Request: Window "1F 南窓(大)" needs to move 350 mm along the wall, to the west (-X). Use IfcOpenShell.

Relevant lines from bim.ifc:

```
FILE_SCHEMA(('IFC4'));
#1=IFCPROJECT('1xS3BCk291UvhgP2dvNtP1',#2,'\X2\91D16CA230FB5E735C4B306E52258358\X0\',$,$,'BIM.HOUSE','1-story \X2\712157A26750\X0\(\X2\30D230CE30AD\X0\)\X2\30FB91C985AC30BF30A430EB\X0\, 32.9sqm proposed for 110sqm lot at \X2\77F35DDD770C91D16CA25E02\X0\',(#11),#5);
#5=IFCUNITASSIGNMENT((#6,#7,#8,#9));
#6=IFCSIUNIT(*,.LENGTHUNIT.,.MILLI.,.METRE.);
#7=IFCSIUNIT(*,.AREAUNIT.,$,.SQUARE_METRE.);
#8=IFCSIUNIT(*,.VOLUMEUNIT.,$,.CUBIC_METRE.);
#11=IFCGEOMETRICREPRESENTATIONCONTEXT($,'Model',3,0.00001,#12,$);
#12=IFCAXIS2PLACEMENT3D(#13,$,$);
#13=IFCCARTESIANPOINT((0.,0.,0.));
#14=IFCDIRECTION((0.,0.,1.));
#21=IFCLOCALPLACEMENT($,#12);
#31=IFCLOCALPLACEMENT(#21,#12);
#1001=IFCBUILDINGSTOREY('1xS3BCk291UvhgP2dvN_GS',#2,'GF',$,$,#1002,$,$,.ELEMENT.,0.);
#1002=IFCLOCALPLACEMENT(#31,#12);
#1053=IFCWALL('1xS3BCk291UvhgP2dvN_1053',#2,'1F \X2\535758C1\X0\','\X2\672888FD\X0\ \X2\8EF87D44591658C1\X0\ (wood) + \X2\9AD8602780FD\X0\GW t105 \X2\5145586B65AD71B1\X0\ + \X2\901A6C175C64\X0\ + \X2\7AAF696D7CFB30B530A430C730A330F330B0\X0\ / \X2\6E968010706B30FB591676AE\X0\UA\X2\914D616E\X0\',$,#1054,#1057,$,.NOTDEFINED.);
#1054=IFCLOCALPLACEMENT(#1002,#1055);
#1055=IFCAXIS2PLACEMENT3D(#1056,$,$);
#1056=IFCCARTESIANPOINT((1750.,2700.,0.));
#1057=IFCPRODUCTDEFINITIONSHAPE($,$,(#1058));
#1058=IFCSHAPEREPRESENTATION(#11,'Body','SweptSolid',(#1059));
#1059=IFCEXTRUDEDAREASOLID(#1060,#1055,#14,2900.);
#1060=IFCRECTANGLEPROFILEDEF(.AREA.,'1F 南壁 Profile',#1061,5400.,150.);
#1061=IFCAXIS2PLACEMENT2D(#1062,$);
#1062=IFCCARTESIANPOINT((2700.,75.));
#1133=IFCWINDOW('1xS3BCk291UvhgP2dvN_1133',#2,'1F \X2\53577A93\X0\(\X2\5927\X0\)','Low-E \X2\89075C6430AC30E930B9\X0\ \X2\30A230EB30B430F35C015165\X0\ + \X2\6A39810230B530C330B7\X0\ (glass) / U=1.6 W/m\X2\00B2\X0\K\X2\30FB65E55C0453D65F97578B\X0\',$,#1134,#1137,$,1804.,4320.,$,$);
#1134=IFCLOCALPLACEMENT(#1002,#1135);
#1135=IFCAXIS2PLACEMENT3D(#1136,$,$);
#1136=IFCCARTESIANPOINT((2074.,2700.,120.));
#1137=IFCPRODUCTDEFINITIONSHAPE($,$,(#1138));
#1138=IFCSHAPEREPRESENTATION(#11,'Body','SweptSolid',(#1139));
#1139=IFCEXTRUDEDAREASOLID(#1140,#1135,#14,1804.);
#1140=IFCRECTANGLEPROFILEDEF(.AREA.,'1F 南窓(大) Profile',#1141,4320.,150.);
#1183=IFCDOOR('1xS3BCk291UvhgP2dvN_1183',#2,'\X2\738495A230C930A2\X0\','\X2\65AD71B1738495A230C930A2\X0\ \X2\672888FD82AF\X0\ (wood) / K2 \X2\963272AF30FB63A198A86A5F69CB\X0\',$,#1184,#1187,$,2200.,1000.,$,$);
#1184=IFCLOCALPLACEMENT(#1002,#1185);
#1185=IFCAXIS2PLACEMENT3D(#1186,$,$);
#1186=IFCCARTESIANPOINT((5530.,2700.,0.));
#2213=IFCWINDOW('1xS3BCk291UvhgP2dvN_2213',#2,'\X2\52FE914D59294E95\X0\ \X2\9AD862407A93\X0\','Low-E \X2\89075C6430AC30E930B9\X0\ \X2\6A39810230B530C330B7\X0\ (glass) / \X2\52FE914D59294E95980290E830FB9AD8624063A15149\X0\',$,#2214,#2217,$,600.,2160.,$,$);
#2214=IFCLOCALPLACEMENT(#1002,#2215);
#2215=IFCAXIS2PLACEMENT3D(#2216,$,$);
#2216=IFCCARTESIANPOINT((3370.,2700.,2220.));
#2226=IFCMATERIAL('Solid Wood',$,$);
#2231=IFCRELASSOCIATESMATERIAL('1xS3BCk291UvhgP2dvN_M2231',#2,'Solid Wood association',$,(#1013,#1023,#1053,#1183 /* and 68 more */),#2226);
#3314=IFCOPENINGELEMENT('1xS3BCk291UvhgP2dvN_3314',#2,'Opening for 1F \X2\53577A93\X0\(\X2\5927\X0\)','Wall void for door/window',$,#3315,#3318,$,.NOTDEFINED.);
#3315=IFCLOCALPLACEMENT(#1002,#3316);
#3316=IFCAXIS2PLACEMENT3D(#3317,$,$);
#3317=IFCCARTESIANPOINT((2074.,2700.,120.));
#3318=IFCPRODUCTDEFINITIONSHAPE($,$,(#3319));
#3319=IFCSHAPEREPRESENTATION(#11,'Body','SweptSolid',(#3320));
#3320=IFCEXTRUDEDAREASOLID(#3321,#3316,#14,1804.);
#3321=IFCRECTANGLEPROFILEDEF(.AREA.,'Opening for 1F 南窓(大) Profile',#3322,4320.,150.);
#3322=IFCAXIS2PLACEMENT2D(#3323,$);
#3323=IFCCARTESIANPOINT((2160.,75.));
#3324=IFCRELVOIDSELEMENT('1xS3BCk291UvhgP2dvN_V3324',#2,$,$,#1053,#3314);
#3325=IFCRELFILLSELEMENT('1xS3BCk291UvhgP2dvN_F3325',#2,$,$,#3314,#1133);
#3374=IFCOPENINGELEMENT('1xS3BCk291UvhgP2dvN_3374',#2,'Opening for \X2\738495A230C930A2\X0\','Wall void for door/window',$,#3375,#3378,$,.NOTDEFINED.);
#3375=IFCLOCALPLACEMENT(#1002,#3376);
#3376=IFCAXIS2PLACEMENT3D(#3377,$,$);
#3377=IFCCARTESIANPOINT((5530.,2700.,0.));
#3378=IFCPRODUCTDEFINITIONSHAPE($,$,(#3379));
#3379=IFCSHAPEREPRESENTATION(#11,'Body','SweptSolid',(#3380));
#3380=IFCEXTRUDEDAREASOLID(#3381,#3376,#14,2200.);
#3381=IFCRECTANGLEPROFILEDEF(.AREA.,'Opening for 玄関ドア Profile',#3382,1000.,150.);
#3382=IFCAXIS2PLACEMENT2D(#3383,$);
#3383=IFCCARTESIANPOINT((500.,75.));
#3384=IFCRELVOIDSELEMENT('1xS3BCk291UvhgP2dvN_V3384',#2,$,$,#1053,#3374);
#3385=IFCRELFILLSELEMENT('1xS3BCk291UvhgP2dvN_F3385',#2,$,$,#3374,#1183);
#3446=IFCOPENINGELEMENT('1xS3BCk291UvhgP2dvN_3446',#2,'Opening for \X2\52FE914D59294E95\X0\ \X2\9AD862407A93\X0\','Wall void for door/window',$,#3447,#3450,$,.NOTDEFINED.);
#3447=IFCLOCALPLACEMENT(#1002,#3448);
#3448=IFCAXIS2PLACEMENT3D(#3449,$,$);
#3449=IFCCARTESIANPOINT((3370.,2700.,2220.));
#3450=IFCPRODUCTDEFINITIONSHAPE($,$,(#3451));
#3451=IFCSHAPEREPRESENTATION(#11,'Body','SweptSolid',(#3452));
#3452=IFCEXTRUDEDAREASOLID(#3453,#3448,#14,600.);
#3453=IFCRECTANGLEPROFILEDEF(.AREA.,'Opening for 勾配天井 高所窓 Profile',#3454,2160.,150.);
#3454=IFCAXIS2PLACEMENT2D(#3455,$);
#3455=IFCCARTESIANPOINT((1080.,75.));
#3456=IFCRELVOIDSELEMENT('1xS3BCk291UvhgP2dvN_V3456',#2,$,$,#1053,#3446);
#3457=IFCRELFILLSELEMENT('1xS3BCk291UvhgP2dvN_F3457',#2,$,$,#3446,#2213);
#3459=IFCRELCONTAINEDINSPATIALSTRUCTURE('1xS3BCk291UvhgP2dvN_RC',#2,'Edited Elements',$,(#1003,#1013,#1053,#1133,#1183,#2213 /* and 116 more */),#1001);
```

```python
import ifcopenshell
import ifcopenshell.api.geometry
import ifcopenshell.util.placement
import ifcopenshell.util.unit

model = ifcopenshell.open("bim.ifc")
unit_scale = ifcopenshell.util.unit.calculate_unit_scale(model)

window = model.by_guid("1xS3BCk291UvhgP2dvN_1133")
opening = window.FillsVoids[0].RelatingOpeningElement
wall = opening.VoidsElements[0].RelatingBuildingElement

wall_matrix = ifcopenshell.util.placement.get_local_placement(wall.ObjectPlacement)
shift = wall_matrix[:3, 0] * -0.35 / unit_scale
before = ifcopenshell.util.placement.get_local_placement(window.ObjectPlacement)[:3, 3].copy()

# The window is not placed relative to its opening, so move both.
for product in (opening, window):
    matrix = ifcopenshell.util.placement.get_local_placement(product.ObjectPlacement)
    matrix[:3, 3] += shift
    ifcopenshell.api.geometry.edit_object_placement(model, product=product, matrix=matrix, is_si=False)

after = ifcopenshell.util.placement.get_local_placement(window.ObjectPlacement)[:3, 3]
print("window moved by", (after - before).round(3) + 0.0)

model.write("bim-out.ifc")
```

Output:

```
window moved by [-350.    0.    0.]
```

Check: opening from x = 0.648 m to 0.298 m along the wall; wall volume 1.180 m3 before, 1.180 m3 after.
